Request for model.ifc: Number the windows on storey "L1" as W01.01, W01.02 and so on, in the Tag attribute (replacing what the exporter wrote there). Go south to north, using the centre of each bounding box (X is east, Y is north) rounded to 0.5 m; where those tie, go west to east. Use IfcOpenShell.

First a look at what the model holds.

```python
import ifcopenshell
import ifcopenshell.util.element
import ifcopenshell.util.placement

model = ifcopenshell.open("model.ifc")
print(model.schema)
storey = next(s for s in model.by_type("IfcBuildingStorey") if s.Name == "L1")
windows = [e for e in ifcopenshell.util.element.get_decomposition(storey) if e.is_a("IfcWindow")]
for e in sorted(windows, key=lambda e: e.id()):
    origin = ifcopenshell.util.placement.get_local_placement(e.ObjectPlacement)[:3, 3]
    print(e.id(), e.Tag, e.Name, origin.round(2) + 0.0, sep=" | ")
```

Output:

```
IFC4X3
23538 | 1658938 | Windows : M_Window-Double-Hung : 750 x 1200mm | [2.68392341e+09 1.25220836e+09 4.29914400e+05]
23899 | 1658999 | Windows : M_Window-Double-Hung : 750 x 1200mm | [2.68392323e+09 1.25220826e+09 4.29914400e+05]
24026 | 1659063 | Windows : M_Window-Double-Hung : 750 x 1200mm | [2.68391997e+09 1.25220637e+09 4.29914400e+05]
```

```python
import ifcopenshell
import ifcopenshell.geom
import ifcopenshell.util.element
import ifcopenshell.util.shape

model = ifcopenshell.open("model.ifc")
settings = ifcopenshell.geom.settings()
settings.set("use-world-coords", True)


def centre(element):
    shape = ifcopenshell.geom.create_shape(settings, element)
    return ifcopenshell.util.shape.get_bbox_centroid(shape.geometry)


storey = next(s for s in model.by_type("IfcBuildingStorey") if s.Name == "L1")
windows = [e for e in ifcopenshell.util.element.get_decomposition(storey) if e.is_a("IfcWindow")]

# Insertion points can sit at a corner or the storey origin, so sort by the geometry (in metres).
centres = {e: centre(e) for e in windows}
windows.sort(key=lambda e: (round(centres[e][1] / 0.5), centres[e][0]))

for i, e in enumerate(windows, start=1):
    number = f"W01.{i:02d}"
    e.Tag = number
    print(e.id(), number)

model.write("model-out.ifc")
```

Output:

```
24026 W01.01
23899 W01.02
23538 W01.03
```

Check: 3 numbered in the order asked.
